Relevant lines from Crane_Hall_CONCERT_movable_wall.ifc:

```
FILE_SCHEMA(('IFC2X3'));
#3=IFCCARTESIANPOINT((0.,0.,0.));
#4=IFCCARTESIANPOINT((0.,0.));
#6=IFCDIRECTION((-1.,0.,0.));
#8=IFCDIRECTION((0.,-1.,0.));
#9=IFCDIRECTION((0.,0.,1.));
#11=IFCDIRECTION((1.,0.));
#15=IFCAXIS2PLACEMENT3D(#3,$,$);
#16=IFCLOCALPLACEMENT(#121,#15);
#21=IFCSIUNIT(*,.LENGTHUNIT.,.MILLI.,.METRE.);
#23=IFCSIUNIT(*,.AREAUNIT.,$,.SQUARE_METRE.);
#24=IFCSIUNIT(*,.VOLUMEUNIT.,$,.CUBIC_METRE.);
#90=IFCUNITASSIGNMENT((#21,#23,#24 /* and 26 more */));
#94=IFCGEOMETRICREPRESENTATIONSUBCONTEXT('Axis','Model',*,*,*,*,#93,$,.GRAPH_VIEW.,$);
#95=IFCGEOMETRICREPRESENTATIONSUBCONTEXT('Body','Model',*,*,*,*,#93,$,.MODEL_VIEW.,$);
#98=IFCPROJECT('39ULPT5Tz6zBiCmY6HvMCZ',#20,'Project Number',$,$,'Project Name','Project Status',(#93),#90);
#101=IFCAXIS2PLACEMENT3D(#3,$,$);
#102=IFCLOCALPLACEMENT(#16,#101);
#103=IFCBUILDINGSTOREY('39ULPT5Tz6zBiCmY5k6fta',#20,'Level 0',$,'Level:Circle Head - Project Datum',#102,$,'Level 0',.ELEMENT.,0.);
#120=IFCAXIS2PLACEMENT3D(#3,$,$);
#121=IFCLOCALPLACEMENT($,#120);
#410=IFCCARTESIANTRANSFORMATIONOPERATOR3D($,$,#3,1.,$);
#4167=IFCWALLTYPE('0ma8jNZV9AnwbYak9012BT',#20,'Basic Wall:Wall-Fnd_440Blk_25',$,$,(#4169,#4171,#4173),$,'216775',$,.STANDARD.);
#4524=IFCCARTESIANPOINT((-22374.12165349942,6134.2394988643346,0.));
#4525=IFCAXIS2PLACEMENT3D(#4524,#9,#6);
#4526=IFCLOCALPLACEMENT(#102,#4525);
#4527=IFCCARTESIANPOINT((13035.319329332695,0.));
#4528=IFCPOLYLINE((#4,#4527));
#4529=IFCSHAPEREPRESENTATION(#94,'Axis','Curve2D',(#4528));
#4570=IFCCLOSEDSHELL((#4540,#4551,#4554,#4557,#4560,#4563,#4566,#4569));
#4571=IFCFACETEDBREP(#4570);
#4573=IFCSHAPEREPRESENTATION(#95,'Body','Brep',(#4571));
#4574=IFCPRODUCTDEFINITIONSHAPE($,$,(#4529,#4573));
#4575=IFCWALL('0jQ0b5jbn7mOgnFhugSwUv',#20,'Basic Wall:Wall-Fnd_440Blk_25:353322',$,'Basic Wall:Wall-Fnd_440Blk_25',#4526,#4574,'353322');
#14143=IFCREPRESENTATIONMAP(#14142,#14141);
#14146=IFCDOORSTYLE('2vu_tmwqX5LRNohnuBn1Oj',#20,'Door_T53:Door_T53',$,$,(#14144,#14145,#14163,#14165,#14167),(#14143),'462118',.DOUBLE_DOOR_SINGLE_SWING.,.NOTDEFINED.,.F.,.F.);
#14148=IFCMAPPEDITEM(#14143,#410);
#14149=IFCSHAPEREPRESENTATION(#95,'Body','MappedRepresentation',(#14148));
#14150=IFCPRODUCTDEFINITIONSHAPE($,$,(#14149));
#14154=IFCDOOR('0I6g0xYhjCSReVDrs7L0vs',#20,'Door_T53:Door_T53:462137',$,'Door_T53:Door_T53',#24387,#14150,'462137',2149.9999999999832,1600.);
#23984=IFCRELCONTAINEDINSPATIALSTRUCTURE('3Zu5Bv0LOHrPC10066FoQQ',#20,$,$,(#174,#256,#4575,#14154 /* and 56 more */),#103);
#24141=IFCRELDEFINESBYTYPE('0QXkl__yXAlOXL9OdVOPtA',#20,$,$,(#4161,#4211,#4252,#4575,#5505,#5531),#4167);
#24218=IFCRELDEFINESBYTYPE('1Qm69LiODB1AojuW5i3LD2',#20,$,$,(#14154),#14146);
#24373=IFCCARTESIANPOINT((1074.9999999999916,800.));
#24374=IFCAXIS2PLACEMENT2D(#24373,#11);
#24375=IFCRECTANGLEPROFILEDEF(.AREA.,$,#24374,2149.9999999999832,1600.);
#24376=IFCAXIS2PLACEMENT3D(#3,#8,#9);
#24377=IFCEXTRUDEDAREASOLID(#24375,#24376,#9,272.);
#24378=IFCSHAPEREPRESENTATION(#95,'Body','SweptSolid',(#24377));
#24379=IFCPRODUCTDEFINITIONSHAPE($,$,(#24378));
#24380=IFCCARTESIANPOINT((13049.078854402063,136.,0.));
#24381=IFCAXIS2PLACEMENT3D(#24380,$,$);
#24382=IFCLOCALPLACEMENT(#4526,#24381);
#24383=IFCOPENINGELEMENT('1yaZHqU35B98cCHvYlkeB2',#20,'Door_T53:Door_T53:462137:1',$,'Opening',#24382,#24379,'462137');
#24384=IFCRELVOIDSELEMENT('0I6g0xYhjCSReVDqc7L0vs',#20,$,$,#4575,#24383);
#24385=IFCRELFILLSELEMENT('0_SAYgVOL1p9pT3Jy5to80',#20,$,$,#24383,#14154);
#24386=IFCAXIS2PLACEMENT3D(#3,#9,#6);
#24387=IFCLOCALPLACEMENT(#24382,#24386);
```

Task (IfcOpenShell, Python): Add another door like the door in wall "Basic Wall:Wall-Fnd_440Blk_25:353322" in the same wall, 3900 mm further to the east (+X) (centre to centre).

```python
import ifcopenshell
import ifcopenshell.api.feature
import ifcopenshell.api.geometry
import ifcopenshell.api.root
import ifcopenshell.geom
import ifcopenshell.util.element
import ifcopenshell.util.placement
import ifcopenshell.util.shape
import ifcopenshell.util.unit

model = ifcopenshell.open("Crane_Hall_CONCERT_movable_wall.ifc")
unit_scale = ifcopenshell.util.unit.calculate_unit_scale(model)
settings = ifcopenshell.geom.settings()


def volume(element):
    """Net volume in cubic metres, openings subtracted."""
    shape = ifcopenshell.geom.create_shape(settings, element)
    return ifcopenshell.util.shape.get_volume(shape.geometry)


def reuse_history(source, copy):
    """copy_class also copies each property set's owner history, people and application; keep the originals."""
    for rel in copy.IsDefinedBy:
        if rel.is_a("IfcRelDefinesByProperties") and (history := rel.RelatingPropertyDefinition.OwnerHistory):
            rel.RelatingPropertyDefinition.OwnerHistory = source.OwnerHistory
            ifcopenshell.util.element.remove_deep2(model, history)


door = model.by_guid("0I6g0xYhjCSReVDrs7L0vs")
opening = door.FillsVoids[0].RelatingOpeningElement
wall = opening.VoidsElements[0].RelatingBuildingElement
before = volume(wall)
shift = ifcopenshell.util.placement.get_local_placement(wall.ObjectPlacement)[:3, 0] * -3.9 / unit_scale

# copy_class copies the void relationship, type, container and properties, but no geometry.
new_opening = ifcopenshell.api.root.copy_class(model, product=opening)
new_opening.Representation = ifcopenshell.util.element.copy_deep(
    model, opening.Representation, exclude=["IfcGeometricRepresentationContext", "IfcRepresentationMap"]
)
new_opening.Name = "Door_T53:Door_T53"
new_opening.Tag = None
new_door = ifcopenshell.api.root.copy_class(model, product=door)
new_door.Representation = ifcopenshell.util.element.copy_deep(
    model, door.Representation, exclude=["IfcGeometricRepresentationContext", "IfcRepresentationMap"]
)
new_door.Name = "Door_T53:Door_T53"
new_door.Tag = None
reuse_history(door, new_door)
fills = ifcopenshell.api.feature.add_filling(model, opening=new_opening, element=new_door)
fills.OwnerHistory = new_door.OwnerHistory  # required in IFC2X3

for old, new in ((opening, new_opening), (door, new_door)):
    matrix = ifcopenshell.util.placement.get_local_placement(old.ObjectPlacement)
    matrix[:3, 3] += shift
    ifcopenshell.api.geometry.edit_object_placement(model, product=new, matrix=matrix, is_si=False)

after = volume(wall)

print(f"wall volume {before:.3f} -> {after:.3f} m3")

model.write("Crane_Hall_CONCERT_movable_wall_updated.ifc")
```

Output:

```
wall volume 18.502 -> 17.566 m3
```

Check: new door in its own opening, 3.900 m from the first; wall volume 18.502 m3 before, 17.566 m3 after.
